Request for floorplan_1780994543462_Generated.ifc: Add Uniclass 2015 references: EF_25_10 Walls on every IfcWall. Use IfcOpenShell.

First a look at what the model holds.

```python
import ifcopenshell

model = ifcopenshell.open("floorplan_1780994543462_Generated.ifc")
print(model.schema)
print("classifications:", [c.Name for c in model.by_type("IfcClassification")])
for ifc_class in ("IfcDoor", "IfcRoof", "IfcStair", "IfcWall", "IfcWindow"):
    print(ifc_class, len(model.by_type(ifc_class)))
```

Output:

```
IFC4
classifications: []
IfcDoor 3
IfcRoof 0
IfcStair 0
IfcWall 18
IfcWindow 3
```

```python
import ifcopenshell
import ifcopenshell.api.classification

model = ifcopenshell.open("floorplan_1780994543462_Generated.ifc")

system = ifcopenshell.api.classification.add_classification(model, classification="Uniclass 2015")

codes = {
    "IfcWall": ("EF_25_10", "Walls"),
}
for ifc_class, (code, name) in codes.items():
    products = model.by_type(ifc_class)
    ifcopenshell.api.classification.add_reference(
        model, products=products, classification=system, identification=code, name=name
    )
    print(code, len(products))

model.write("floorplan_1780994543462_Generated_edited.ifc")
```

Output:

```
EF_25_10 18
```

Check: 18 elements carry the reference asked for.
